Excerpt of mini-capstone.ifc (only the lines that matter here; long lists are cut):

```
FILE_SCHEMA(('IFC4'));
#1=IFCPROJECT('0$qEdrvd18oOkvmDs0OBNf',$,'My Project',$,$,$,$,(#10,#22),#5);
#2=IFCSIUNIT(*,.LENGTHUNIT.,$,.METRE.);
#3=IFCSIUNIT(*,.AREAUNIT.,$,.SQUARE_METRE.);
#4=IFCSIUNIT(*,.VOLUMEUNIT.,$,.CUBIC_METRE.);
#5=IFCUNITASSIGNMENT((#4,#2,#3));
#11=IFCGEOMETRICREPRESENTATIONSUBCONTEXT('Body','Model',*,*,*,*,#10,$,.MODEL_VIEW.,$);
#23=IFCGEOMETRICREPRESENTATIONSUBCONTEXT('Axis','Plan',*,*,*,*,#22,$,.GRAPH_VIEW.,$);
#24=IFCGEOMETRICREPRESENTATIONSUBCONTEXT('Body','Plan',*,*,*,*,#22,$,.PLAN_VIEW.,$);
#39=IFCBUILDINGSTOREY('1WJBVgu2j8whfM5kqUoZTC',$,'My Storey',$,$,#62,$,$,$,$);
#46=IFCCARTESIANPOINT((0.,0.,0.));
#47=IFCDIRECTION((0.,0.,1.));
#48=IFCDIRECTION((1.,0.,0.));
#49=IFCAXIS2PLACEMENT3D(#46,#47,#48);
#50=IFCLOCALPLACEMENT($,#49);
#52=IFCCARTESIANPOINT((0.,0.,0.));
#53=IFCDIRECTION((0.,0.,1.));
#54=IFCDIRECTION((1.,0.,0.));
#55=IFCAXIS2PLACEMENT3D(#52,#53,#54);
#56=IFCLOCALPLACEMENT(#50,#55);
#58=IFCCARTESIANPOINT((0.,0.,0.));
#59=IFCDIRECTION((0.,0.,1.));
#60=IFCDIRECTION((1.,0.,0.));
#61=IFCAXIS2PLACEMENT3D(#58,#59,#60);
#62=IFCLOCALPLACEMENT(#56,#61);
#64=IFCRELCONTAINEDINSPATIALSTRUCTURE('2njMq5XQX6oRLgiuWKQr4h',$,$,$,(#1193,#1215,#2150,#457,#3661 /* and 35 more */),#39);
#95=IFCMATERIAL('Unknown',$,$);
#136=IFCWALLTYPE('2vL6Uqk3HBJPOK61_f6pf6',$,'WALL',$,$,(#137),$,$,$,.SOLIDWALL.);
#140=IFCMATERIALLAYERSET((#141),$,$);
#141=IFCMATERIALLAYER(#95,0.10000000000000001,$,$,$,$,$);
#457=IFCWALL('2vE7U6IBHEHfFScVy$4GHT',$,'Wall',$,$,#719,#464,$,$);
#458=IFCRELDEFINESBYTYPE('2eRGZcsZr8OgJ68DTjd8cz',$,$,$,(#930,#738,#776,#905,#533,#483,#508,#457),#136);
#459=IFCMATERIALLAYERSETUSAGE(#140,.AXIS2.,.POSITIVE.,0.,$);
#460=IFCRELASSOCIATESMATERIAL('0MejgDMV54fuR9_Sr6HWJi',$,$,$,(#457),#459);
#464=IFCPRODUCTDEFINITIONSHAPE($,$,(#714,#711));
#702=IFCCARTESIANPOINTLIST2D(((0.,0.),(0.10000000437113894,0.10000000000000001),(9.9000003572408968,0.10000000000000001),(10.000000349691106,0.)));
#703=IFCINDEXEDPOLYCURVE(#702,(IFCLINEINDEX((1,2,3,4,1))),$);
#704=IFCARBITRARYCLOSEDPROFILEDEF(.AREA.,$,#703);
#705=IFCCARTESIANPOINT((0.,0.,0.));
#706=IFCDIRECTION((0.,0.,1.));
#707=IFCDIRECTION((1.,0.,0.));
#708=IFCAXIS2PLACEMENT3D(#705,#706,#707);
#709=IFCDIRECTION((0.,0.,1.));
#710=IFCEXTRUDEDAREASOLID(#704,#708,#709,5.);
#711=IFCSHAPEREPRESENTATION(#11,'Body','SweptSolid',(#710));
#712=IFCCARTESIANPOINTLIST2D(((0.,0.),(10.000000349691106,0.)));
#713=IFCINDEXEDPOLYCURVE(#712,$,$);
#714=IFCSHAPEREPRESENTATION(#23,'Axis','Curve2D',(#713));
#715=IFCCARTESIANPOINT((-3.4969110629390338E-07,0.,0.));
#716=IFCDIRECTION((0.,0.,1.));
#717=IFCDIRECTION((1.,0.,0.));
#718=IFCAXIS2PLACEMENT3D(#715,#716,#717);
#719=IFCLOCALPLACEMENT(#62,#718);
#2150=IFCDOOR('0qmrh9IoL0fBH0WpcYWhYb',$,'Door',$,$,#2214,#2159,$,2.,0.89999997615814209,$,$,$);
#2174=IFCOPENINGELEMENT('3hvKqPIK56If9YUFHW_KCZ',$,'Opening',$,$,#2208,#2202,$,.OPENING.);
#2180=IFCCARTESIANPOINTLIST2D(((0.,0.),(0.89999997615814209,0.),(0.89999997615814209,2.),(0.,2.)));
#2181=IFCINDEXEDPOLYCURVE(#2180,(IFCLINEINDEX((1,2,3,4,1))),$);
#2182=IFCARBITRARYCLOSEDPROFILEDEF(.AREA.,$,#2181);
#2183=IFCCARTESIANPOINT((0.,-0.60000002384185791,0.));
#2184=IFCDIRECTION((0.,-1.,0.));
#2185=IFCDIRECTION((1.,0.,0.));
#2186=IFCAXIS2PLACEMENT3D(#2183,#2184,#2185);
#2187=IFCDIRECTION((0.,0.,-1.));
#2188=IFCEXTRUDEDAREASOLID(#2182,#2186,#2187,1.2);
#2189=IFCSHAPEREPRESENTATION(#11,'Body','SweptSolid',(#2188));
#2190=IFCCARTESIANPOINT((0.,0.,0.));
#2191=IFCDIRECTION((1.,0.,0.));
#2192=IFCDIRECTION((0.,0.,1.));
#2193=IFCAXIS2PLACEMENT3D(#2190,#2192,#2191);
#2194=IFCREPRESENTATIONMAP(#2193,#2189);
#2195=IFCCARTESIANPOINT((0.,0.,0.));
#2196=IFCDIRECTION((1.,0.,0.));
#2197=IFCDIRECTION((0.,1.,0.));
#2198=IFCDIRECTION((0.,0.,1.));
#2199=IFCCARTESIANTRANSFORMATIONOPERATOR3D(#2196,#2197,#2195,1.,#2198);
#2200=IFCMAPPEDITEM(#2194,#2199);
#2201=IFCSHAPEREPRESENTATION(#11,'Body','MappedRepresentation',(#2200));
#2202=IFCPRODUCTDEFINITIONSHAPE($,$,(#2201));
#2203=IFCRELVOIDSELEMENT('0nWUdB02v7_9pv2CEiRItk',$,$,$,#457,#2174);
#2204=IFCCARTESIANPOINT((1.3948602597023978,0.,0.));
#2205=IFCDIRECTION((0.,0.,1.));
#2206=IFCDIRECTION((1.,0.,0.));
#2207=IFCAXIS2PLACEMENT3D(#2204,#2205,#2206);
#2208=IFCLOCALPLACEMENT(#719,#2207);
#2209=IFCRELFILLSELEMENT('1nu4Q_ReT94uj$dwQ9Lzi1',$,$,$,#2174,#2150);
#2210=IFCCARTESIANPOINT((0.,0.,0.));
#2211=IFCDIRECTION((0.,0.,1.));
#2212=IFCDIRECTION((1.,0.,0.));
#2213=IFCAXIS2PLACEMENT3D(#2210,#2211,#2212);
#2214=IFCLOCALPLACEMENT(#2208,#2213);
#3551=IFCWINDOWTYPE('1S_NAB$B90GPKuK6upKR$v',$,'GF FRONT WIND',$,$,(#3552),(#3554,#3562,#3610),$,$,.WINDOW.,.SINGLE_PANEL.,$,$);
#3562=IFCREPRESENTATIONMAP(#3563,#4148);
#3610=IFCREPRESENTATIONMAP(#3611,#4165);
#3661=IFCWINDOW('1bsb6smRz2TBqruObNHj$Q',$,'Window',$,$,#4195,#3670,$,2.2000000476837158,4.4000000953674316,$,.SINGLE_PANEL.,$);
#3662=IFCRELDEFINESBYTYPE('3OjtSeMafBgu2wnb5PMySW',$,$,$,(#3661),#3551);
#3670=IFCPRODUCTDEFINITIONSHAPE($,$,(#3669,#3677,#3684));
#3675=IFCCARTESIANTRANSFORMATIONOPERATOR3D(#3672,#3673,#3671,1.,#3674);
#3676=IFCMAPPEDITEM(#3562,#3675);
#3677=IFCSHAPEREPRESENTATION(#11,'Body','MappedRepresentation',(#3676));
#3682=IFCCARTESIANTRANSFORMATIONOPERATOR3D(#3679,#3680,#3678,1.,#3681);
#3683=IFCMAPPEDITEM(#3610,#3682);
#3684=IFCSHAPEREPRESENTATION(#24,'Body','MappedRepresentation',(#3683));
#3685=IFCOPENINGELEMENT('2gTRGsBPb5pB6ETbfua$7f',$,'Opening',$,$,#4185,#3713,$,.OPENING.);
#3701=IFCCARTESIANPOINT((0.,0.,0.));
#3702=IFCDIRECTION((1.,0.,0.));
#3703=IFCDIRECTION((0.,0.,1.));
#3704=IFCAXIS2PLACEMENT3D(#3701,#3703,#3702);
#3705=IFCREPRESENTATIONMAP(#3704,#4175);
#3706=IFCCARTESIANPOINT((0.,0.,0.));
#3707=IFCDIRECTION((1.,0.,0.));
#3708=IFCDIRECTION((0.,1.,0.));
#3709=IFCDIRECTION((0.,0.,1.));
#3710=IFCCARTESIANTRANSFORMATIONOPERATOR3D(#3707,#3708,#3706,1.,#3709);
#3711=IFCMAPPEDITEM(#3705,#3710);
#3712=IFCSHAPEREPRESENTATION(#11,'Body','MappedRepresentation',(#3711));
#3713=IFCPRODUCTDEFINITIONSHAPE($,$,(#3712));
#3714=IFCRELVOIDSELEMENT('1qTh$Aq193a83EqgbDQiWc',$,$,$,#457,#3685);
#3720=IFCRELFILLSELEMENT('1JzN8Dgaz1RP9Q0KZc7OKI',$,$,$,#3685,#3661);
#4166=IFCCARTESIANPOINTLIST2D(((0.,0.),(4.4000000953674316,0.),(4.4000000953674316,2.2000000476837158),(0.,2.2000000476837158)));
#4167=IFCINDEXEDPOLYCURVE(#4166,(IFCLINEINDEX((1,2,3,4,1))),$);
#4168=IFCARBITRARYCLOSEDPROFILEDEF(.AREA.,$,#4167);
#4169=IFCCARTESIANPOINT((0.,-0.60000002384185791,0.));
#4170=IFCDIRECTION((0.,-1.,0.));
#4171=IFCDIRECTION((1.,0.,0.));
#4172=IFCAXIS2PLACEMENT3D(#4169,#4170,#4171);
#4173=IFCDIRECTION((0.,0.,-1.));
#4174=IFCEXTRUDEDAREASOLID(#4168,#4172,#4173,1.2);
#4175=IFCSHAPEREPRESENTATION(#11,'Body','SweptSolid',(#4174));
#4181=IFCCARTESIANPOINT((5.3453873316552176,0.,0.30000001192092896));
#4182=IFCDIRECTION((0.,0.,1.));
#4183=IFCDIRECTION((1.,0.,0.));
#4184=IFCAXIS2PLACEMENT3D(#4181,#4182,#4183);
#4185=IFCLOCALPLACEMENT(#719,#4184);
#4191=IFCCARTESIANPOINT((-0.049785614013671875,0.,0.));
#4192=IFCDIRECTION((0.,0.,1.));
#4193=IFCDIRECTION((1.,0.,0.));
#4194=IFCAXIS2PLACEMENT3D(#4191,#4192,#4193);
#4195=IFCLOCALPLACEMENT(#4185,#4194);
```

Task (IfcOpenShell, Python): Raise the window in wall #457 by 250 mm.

```python
import numpy as np
import ifcopenshell
import ifcopenshell.api.geometry
import ifcopenshell.util.placement
import ifcopenshell.util.unit

model = ifcopenshell.open("mini-capstone.ifc")
unit_scale = ifcopenshell.util.unit.calculate_unit_scale(model)

window = model.by_guid("1bsb6smRz2TBqruObNHj$Q")
opening = window.FillsVoids[0].RelatingOpeningElement
dz = 0.25 / unit_scale

shift = np.array([0.0, 0.0, dz])
# The window is placed relative to its opening, so it follows when the opening moves.
matrix = ifcopenshell.util.placement.get_local_placement(opening.ObjectPlacement)
matrix[:3, 3] += shift
ifcopenshell.api.geometry.edit_object_placement(
    model, product=opening, matrix=matrix, is_si=False, should_transform_children=True
)

print(f"moved by {dz * unit_scale:+.3f} m")

model.write("mini-capstone_updated.ifc")
```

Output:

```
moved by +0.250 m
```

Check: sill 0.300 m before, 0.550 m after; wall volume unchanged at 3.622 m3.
